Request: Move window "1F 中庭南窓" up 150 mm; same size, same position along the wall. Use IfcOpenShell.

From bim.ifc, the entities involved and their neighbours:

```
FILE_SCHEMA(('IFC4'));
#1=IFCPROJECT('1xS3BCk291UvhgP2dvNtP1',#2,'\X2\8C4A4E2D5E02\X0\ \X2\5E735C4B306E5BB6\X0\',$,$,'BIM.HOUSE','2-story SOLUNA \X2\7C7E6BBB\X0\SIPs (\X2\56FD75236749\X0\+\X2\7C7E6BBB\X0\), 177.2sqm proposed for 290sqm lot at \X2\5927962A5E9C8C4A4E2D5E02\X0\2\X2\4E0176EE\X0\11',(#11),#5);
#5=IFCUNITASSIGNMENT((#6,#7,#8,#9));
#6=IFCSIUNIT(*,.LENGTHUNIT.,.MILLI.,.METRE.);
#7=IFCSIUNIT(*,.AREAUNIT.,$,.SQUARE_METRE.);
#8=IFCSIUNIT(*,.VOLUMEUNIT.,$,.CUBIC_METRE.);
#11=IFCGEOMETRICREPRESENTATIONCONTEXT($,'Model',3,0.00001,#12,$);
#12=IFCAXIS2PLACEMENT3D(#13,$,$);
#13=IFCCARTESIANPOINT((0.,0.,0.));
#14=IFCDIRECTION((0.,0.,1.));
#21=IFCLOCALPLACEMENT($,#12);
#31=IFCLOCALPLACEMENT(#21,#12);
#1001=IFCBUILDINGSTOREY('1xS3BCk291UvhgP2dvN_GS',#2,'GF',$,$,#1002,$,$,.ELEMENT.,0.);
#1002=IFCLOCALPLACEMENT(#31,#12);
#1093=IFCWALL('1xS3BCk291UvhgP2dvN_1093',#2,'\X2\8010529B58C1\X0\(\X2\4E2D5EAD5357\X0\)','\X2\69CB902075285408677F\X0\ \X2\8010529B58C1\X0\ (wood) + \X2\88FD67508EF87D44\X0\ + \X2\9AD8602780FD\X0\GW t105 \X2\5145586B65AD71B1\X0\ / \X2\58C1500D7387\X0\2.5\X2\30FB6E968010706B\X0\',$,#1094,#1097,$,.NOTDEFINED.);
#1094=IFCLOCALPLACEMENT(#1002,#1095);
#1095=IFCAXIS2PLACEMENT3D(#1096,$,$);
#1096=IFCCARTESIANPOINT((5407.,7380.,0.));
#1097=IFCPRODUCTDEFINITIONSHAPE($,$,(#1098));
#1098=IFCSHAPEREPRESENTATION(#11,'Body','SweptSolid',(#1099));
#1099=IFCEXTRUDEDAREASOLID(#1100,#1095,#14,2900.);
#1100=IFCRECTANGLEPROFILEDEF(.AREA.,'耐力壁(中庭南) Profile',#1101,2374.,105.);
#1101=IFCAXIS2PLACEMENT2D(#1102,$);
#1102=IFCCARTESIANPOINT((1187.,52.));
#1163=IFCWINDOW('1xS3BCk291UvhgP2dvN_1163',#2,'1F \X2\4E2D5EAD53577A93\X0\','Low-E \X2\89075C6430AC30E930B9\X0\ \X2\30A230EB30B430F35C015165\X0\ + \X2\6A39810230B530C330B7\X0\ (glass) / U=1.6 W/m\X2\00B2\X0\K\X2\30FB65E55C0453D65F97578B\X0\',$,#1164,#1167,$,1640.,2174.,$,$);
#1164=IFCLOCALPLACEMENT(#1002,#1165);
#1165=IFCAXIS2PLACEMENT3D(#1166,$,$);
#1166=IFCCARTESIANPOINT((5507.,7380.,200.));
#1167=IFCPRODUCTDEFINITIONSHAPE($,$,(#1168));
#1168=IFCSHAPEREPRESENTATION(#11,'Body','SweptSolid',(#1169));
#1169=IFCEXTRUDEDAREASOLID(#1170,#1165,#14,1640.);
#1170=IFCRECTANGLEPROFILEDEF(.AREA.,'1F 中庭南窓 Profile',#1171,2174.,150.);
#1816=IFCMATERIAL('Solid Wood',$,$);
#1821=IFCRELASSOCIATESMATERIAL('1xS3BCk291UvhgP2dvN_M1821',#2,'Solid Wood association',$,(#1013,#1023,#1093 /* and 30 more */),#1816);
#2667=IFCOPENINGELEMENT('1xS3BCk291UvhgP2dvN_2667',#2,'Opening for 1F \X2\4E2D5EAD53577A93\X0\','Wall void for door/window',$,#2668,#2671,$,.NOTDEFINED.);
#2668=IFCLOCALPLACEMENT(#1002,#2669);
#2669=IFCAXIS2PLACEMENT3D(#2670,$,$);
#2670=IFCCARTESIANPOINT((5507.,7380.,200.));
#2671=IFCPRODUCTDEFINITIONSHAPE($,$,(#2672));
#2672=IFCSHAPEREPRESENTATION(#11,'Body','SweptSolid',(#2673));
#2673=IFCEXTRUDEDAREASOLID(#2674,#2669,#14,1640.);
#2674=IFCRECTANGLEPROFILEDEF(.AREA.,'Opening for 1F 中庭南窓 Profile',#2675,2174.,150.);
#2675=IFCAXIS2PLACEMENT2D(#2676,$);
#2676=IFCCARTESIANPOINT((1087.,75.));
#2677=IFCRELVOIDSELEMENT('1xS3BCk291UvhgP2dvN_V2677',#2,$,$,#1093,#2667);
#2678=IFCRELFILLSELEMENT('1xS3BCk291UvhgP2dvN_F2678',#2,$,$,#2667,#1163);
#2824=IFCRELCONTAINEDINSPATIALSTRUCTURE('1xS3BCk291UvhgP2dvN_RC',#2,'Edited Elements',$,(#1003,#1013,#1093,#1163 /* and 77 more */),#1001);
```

```python
import numpy as np
import ifcopenshell
import ifcopenshell.api.geometry
import ifcopenshell.util.placement
import ifcopenshell.util.unit

model = ifcopenshell.open("bim.ifc")
unit_scale = ifcopenshell.util.unit.calculate_unit_scale(model)

window = model.by_guid("1xS3BCk291UvhgP2dvN_1163")
opening = window.FillsVoids[0].RelatingOpeningElement
dz = 0.15 / unit_scale

shift = np.array([0.0, 0.0, dz])
# The window is not placed relative to its opening, so move both.
for product in (opening, window):
    matrix = ifcopenshell.util.placement.get_local_placement(product.ObjectPlacement)
    matrix[:3, 3] += shift
    ifcopenshell.api.geometry.edit_object_placement(model, product=product, matrix=matrix, is_si=False)

print(f"moved by {dz * unit_scale:+.3f} m")

model.write("bim_v2.ifc")
```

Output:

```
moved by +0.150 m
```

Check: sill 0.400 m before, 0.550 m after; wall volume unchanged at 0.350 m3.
